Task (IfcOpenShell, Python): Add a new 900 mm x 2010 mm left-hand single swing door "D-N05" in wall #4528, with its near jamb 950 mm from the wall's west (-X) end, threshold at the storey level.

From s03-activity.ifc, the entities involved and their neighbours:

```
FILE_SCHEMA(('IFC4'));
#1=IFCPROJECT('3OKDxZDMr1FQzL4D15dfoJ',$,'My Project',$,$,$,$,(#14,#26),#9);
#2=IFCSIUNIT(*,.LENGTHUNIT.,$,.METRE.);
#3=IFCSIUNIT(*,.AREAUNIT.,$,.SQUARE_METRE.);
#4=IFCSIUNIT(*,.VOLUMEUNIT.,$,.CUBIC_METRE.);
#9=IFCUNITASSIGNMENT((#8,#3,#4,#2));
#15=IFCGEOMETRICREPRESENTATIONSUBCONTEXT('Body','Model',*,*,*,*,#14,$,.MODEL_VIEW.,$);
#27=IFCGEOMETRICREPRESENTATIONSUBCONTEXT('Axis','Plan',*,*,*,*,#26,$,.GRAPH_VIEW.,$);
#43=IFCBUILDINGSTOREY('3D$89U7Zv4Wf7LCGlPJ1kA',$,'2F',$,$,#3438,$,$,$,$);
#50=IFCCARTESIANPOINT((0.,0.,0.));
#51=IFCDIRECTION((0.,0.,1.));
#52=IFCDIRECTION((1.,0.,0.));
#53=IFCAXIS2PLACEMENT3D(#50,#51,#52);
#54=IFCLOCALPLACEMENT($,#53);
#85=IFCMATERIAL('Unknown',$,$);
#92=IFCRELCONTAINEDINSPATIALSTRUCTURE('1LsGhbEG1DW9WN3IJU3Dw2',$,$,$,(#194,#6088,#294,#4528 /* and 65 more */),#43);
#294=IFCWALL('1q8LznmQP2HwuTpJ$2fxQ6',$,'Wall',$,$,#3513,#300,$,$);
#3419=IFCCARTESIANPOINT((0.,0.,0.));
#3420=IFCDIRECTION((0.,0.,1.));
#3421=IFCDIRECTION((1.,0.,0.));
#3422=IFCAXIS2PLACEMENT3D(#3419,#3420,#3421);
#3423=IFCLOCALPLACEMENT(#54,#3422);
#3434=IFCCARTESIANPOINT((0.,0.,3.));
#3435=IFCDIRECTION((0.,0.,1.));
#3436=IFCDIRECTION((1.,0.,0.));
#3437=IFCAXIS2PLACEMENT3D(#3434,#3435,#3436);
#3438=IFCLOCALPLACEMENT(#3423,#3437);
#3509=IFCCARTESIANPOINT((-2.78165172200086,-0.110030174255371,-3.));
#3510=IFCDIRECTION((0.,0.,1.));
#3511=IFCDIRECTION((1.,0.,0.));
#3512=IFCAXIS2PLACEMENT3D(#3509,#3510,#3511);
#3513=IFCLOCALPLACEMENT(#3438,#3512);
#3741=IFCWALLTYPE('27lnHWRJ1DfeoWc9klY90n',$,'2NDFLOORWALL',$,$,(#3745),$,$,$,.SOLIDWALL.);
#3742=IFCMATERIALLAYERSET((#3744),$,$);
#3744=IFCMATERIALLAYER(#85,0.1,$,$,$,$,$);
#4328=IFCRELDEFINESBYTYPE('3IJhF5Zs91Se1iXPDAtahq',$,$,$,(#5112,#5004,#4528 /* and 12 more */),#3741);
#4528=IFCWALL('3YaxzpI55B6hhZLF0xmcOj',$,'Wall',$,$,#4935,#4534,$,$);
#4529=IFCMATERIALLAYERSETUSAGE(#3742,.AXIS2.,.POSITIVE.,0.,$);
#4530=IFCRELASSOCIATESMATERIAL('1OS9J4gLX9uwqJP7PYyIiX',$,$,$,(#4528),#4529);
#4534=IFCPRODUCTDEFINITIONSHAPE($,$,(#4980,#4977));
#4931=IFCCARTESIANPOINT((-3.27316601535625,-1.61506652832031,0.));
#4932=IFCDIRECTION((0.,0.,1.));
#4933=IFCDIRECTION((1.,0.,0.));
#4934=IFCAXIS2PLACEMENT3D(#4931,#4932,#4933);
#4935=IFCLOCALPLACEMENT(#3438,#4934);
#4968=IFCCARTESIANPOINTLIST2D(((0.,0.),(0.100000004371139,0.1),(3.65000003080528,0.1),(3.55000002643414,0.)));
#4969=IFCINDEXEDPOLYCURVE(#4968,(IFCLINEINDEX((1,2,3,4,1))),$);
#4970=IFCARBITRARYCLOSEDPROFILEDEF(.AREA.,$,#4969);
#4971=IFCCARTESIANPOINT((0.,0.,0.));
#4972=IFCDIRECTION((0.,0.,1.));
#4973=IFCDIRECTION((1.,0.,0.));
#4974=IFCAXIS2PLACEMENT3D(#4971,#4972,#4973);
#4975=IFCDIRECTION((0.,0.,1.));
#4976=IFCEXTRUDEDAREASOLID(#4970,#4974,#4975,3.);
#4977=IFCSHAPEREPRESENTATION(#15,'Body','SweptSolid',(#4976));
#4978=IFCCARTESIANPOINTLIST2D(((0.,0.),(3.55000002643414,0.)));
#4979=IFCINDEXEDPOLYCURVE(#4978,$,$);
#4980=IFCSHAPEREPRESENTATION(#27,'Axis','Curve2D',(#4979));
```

```python
import numpy as np
import ifcopenshell
import ifcopenshell.api.feature
import ifcopenshell.api.geometry
import ifcopenshell.api.root
import ifcopenshell.api.spatial
import ifcopenshell.geom
import ifcopenshell.util.element
import ifcopenshell.util.placement
import ifcopenshell.util.representation
import ifcopenshell.util.shape
import ifcopenshell.util.unit

model = ifcopenshell.open("s03-activity.ifc")
unit_scale = ifcopenshell.util.unit.calculate_unit_scale(model)
settings = ifcopenshell.geom.settings()


def volume(element):
    """Net volume in cubic metres, openings subtracted."""
    shape = ifcopenshell.geom.create_shape(settings, element)
    return ifcopenshell.util.shape.get_volume(shape.geometry)


wall = model.by_id(4528)
storey = ifcopenshell.util.element.get_container(wall, ifc_class="IfcBuildingStorey")
context = ifcopenshell.util.representation.get_context(model, "Model", "Body", "MODEL_VIEW")
before = volume(wall)

width, height, from_end, sill = 0.9, 2.01, 0.95, 0.0  # metres

# The wall runs along its own X axis, and the end named is its -X end.
wall_shape = ifcopenshell.geom.create_shape(settings, wall)
x, y, z = ifcopenshell.util.shape.get_vertices(wall_shape.geometry).T
start = x.min() + from_end
face, thickness = float(y.min()), float(y.max() - y.min())
wall_matrix = ifcopenshell.util.placement.get_local_placement(wall.ObjectPlacement)
level = ifcopenshell.util.placement.get_local_placement(storey.ObjectPlacement)[2, 3]


def in_wall(x, y):
    """Placement at x, y metres in the wall's axes, at sill height."""
    matrix = wall_matrix.copy()
    matrix[:, 3] = wall_matrix @ np.array([x / unit_scale, y / unit_scale, 0.0, 1.0])
    matrix[2, 3] = level + sill / unit_scale
    return matrix


# Opening: a box that overshoots both wall faces by 50 mm.
opening = ifcopenshell.api.root.create_entity(model, ifc_class="IfcOpeningElement", predefined_type="OPENING")
box = ifcopenshell.api.geometry.add_wall_representation(
    model, context=context, length=width, height=height, thickness=thickness + 0.1
)
ifcopenshell.api.geometry.assign_representation(model, product=opening, representation=box)
ifcopenshell.api.geometry.edit_object_placement(model, product=opening, matrix=in_wall(start, face - 0.05), is_si=False)
ifcopenshell.api.feature.add_feature(model, feature=opening, element=wall)

door = ifcopenshell.api.root.create_entity(model, ifc_class="IfcDoor", name="D-N05", predefined_type="DOOR")
door.OverallWidth, door.OverallHeight = width / unit_scale, height / unit_scale
door.OperationType = "SINGLE_SWING_LEFT"
body = ifcopenshell.api.geometry.add_door_representation(
    model,
    context=context,
    overall_width=door.OverallWidth,
    overall_height=door.OverallHeight,
    operation_type="SINGLE_SWING_LEFT",
    lining_properties={"LiningDepth": thickness / unit_scale, "ThresholdDepth": thickness / unit_scale},
)
ifcopenshell.api.geometry.assign_representation(model, product=door, representation=body)
ifcopenshell.api.spatial.assign_container(model, products=[door], relating_structure=storey)
ifcopenshell.api.feature.add_filling(model, opening=opening, element=door)

# The lining spans the wall, so the door starts at the wall face.
ifcopenshell.api.geometry.edit_object_placement(model, product=door, matrix=in_wall(start, face), is_si=False)

after = volume(wall)

print(f"wall volume {before:.3f} -> {after:.3f} m3")

model.write("s03-activity_v2.ifc")
```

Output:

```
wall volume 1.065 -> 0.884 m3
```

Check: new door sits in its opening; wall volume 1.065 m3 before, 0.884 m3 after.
